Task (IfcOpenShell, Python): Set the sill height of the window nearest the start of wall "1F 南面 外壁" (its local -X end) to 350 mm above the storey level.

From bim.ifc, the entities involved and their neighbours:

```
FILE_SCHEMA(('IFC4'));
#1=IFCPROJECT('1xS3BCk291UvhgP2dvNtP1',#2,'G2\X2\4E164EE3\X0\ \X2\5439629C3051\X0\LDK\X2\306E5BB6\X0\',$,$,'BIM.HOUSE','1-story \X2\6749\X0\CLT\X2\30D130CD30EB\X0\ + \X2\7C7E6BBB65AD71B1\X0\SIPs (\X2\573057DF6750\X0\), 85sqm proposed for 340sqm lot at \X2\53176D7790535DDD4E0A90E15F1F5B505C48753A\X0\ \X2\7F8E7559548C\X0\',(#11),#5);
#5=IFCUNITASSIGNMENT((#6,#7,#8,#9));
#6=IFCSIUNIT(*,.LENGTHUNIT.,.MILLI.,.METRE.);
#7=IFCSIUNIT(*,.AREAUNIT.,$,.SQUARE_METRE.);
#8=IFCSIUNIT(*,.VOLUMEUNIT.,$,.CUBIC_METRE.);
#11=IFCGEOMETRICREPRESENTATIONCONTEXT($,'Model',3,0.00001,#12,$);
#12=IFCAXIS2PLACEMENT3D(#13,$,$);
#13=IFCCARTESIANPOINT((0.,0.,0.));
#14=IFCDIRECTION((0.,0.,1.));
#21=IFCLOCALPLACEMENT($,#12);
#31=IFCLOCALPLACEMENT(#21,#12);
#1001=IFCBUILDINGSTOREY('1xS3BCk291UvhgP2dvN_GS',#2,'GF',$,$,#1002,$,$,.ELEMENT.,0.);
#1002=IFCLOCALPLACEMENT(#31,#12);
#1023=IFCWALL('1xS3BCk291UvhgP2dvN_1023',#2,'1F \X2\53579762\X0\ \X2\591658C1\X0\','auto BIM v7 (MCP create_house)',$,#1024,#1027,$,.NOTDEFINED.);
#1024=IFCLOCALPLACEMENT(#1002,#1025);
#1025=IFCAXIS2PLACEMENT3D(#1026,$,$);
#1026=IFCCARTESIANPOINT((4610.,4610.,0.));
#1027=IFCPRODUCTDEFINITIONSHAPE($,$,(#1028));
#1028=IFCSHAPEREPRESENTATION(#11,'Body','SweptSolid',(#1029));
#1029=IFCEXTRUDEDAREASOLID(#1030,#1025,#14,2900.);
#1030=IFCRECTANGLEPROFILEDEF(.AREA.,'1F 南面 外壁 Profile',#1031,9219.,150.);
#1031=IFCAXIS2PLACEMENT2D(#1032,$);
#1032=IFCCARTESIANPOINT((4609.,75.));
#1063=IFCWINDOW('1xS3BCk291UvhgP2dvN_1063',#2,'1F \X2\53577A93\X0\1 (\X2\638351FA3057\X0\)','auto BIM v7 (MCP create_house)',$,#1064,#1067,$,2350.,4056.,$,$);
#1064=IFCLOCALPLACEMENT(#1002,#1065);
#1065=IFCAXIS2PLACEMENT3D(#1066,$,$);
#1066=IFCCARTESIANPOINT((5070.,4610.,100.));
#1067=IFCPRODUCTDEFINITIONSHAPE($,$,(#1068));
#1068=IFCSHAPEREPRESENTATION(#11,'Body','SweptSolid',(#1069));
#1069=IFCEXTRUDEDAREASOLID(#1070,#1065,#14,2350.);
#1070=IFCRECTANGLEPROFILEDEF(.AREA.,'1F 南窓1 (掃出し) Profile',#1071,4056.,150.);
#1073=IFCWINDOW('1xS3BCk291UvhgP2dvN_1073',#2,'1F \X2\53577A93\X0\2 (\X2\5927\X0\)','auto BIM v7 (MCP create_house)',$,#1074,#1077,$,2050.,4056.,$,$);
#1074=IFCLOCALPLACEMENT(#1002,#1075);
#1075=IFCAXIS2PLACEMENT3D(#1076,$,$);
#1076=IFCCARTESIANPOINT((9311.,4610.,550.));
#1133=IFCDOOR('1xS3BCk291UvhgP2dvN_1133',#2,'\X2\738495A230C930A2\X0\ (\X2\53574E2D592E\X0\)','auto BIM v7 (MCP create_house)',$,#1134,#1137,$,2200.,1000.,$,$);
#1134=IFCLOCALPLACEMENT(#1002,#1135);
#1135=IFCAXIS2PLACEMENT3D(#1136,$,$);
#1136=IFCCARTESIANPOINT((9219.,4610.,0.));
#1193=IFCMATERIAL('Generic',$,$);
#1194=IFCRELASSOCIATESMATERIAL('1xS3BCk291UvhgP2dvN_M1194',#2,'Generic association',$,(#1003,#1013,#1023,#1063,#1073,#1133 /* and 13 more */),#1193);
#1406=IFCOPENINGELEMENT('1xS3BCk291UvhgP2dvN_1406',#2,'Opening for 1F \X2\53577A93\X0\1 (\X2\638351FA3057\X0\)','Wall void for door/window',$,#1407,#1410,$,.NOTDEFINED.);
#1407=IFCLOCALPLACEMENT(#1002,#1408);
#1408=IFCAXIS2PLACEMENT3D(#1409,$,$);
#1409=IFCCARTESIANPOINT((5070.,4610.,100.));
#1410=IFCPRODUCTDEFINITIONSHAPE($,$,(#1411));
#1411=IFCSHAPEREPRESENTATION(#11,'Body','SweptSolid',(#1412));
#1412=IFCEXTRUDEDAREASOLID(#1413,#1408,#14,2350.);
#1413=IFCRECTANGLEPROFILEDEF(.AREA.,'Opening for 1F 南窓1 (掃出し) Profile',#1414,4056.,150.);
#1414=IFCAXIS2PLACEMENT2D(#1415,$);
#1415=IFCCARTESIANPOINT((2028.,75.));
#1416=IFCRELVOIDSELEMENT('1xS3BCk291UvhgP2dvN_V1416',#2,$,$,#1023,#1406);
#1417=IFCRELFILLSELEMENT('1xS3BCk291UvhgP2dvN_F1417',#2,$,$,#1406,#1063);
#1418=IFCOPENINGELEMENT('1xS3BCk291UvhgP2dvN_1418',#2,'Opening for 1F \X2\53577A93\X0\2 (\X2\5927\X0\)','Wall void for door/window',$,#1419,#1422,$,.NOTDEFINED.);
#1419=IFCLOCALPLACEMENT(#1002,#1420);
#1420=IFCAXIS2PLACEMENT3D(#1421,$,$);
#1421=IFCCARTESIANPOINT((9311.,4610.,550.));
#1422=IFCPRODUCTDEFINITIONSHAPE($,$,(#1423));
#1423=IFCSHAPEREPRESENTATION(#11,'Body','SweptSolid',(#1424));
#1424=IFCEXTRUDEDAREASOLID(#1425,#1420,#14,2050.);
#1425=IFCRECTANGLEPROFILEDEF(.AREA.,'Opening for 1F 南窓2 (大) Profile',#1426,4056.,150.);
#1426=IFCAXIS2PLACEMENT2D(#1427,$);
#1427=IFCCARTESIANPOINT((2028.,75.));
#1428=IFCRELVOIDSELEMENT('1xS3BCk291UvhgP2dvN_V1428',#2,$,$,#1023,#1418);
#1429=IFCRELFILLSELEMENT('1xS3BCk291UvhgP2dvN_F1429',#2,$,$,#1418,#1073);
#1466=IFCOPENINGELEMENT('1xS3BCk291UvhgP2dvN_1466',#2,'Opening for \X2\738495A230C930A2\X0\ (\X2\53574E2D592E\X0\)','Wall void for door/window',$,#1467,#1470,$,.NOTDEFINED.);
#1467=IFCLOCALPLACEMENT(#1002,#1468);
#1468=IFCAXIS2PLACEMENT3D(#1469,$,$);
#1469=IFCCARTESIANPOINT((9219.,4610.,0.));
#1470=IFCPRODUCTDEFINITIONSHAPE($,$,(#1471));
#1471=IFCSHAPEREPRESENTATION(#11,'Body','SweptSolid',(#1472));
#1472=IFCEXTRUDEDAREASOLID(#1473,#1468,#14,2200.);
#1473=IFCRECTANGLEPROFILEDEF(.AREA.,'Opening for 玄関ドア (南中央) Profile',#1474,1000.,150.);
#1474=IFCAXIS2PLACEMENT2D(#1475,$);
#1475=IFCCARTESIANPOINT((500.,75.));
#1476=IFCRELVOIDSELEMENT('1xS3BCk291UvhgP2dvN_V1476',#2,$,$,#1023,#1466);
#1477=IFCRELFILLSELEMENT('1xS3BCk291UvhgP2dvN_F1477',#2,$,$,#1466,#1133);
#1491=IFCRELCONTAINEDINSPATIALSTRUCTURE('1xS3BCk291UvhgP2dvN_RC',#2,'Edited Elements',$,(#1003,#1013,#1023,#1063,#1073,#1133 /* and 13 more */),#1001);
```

```python
import numpy as np
import ifcopenshell
import ifcopenshell.api.geometry
import ifcopenshell.geom
import ifcopenshell.util.element
import ifcopenshell.util.placement
import ifcopenshell.util.shape
import ifcopenshell.util.unit

model = ifcopenshell.open("bim.ifc")
unit_scale = ifcopenshell.util.unit.calculate_unit_scale(model)

window = model.by_id(1063)
opening = window.FillsVoids[0].RelatingOpeningElement
storey = ifcopenshell.util.element.get_container(window, ifc_class="IfcBuildingStorey")
level = ifcopenshell.util.placement.get_local_placement(storey.ObjectPlacement)[2, 3]

# The opening's origin need not be at the sill, so measure its lowest point.
shape = ifcopenshell.geom.create_shape(ifcopenshell.geom.settings(), opening)
bottom = ifcopenshell.util.shape.get_shape_bottom_elevation(shape, shape.geometry) / unit_scale
dz = level + 0.35 / unit_scale - bottom

shift = np.array([0.0, 0.0, dz])
# The window is not placed relative to its opening, so move both.
for product in (opening, window):
    matrix = ifcopenshell.util.placement.get_local_placement(product.ObjectPlacement)
    matrix[:3, 3] += shift
    ifcopenshell.api.geometry.edit_object_placement(model, product=product, matrix=matrix, is_si=False)

print(f"moved by {dz * unit_scale:+.3f} m")

model.write("bim_edited.ifc")
```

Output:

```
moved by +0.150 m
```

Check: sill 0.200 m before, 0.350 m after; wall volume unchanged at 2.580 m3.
